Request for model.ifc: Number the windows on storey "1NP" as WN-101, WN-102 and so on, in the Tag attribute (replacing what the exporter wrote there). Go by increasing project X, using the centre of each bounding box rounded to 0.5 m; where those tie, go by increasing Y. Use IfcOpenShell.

First a look at what the model holds.

```python
import ifcopenshell
import ifcopenshell.util.element
import ifcopenshell.util.placement

model = ifcopenshell.open("model.ifc")
print(model.schema)
storey = next(s for s in model.by_type("IfcBuildingStorey") if s.Name == "1NP")
windows = [e for e in ifcopenshell.util.element.get_decomposition(storey) if e.is_a("IfcWindow")]
for e in sorted(windows, key=lambda e: e.id()):
    origin = ifcopenshell.util.placement.get_local_placement(e.ObjectPlacement)[:3, 3]
    print(e.id(), e.Tag, e.Name, origin.round(2) + 0.0, sep=" | ")
```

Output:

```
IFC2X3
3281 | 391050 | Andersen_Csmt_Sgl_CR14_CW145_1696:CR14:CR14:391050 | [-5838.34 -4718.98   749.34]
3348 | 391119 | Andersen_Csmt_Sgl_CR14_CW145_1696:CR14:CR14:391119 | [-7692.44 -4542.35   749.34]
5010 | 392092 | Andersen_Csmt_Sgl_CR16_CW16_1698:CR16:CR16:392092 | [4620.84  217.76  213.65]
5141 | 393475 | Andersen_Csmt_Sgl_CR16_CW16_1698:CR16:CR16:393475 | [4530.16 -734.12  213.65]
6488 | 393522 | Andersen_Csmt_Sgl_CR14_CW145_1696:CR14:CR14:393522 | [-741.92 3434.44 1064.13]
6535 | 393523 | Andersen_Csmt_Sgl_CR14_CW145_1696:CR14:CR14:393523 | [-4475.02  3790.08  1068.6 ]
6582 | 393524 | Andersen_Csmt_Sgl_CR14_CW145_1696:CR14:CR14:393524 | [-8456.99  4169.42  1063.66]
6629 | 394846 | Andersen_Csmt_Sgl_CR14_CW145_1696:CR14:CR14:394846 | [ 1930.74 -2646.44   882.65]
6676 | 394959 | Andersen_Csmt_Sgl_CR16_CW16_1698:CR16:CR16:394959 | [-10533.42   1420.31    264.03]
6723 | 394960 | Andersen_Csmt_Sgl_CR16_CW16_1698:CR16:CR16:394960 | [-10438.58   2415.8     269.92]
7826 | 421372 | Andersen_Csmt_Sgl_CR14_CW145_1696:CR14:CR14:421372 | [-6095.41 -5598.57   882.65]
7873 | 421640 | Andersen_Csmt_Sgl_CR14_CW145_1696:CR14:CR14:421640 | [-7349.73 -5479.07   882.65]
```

```python
import ifcopenshell
import ifcopenshell.geom
import ifcopenshell.util.element
import ifcopenshell.util.shape

model = ifcopenshell.open("model.ifc")
settings = ifcopenshell.geom.settings()
settings.set("use-world-coords", True)


def centre(element):
    shape = ifcopenshell.geom.create_shape(settings, element)
    return ifcopenshell.util.shape.get_bbox_centroid(shape.geometry)


storey = next(s for s in model.by_type("IfcBuildingStorey") if s.Name == "1NP")
windows = [e for e in ifcopenshell.util.element.get_decomposition(storey) if e.is_a("IfcWindow")]

# Insertion points can sit at a corner or the storey origin, so sort by the geometry (in metres).
centres = {e: centre(e) for e in windows}
windows.sort(key=lambda e: (round(centres[e][0] / 0.5), centres[e][1]))

for i, e in enumerate(windows, start=1):
    number = f"WN-1{i:02d}"
    e.Tag = number
    print(e.id(), number)

model.write("model_rev.ifc")
```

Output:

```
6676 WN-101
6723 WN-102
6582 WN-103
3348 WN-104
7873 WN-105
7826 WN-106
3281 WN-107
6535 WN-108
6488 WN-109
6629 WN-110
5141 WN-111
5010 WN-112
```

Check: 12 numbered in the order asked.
